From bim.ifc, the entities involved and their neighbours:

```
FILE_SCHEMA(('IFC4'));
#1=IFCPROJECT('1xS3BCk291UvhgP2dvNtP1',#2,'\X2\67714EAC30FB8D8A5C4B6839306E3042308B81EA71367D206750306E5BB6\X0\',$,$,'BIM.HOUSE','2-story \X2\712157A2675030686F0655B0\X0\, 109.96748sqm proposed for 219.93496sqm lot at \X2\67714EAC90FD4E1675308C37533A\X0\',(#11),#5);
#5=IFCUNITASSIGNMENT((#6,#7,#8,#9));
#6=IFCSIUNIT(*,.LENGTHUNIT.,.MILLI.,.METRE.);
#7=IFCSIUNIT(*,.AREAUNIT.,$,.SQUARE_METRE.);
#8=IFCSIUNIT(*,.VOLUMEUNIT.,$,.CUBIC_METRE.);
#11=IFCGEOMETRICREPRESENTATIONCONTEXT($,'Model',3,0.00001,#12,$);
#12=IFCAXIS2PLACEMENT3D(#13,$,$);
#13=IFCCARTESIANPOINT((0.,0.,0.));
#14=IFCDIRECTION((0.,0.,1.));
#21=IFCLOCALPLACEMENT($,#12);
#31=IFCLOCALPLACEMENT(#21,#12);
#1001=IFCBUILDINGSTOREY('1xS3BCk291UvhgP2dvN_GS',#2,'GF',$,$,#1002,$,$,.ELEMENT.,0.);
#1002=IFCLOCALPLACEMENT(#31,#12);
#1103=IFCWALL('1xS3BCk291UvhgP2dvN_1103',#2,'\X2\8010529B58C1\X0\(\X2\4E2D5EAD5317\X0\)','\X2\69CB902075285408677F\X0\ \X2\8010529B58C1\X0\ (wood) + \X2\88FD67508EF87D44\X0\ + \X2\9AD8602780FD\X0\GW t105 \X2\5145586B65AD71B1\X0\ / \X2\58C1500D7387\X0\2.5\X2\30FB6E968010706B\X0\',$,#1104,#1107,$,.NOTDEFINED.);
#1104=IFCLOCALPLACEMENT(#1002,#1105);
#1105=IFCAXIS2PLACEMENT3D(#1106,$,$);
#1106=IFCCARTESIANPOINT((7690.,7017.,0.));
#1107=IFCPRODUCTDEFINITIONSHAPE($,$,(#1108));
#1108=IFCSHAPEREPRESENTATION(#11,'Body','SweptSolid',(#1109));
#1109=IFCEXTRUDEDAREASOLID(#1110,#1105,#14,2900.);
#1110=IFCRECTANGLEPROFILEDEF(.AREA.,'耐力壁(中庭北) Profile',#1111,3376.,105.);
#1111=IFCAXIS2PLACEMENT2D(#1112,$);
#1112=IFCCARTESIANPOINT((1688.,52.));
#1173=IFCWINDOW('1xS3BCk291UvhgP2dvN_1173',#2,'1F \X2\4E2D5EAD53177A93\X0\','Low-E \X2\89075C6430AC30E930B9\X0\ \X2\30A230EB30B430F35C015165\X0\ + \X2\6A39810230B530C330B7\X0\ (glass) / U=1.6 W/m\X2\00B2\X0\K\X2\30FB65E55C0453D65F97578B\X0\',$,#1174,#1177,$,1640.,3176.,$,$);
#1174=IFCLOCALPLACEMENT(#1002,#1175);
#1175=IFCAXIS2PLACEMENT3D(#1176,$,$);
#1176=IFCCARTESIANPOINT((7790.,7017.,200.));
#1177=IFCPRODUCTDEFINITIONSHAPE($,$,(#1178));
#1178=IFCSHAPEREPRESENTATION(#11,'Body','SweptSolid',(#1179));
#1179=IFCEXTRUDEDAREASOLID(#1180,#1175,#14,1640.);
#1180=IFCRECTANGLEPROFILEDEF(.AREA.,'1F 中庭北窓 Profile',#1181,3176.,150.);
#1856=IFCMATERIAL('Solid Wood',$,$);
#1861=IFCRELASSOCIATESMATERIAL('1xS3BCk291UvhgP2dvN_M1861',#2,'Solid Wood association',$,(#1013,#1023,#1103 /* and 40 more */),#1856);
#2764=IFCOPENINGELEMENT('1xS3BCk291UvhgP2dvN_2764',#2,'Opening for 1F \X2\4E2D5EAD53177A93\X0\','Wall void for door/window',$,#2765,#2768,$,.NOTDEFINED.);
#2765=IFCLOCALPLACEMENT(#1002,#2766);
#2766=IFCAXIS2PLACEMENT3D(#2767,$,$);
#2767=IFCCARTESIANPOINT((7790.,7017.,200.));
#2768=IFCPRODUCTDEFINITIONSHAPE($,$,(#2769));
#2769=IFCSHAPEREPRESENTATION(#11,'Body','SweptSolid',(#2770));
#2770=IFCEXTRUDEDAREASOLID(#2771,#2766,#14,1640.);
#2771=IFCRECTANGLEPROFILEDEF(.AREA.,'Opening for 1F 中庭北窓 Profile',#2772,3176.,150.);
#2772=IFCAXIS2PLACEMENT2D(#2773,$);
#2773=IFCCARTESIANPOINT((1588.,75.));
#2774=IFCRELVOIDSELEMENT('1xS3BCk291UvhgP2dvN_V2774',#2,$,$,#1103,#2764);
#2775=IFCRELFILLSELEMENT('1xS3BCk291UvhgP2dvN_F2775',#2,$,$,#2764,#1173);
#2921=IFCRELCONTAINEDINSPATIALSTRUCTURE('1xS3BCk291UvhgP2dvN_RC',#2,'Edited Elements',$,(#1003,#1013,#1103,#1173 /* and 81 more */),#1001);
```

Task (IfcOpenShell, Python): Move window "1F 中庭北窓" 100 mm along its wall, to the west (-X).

```python
import ifcopenshell
import ifcopenshell.api.geometry
import ifcopenshell.util.placement
import ifcopenshell.util.unit

model = ifcopenshell.open("bim.ifc")
unit_scale = ifcopenshell.util.unit.calculate_unit_scale(model)

window = model.by_guid("1xS3BCk291UvhgP2dvN_1173")
opening = window.FillsVoids[0].RelatingOpeningElement
wall = opening.VoidsElements[0].RelatingBuildingElement

wall_matrix = ifcopenshell.util.placement.get_local_placement(wall.ObjectPlacement)
shift = wall_matrix[:3, 0] * -0.1 / unit_scale
before = ifcopenshell.util.placement.get_local_placement(window.ObjectPlacement)[:3, 3].copy()

# The window is not placed relative to its opening, so move both.
for product in (opening, window):
    matrix = ifcopenshell.util.placement.get_local_placement(product.ObjectPlacement)
    matrix[:3, 3] += shift
    ifcopenshell.api.geometry.edit_object_placement(model, product=product, matrix=matrix, is_si=False)

after = ifcopenshell.util.placement.get_local_placement(window.ObjectPlacement)[:3, 3]
print("window moved by", (after - before).round(3) + 0.0)

model.write("bim_updated.ifc")
```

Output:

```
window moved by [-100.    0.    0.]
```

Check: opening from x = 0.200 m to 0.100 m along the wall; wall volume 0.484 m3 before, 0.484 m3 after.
